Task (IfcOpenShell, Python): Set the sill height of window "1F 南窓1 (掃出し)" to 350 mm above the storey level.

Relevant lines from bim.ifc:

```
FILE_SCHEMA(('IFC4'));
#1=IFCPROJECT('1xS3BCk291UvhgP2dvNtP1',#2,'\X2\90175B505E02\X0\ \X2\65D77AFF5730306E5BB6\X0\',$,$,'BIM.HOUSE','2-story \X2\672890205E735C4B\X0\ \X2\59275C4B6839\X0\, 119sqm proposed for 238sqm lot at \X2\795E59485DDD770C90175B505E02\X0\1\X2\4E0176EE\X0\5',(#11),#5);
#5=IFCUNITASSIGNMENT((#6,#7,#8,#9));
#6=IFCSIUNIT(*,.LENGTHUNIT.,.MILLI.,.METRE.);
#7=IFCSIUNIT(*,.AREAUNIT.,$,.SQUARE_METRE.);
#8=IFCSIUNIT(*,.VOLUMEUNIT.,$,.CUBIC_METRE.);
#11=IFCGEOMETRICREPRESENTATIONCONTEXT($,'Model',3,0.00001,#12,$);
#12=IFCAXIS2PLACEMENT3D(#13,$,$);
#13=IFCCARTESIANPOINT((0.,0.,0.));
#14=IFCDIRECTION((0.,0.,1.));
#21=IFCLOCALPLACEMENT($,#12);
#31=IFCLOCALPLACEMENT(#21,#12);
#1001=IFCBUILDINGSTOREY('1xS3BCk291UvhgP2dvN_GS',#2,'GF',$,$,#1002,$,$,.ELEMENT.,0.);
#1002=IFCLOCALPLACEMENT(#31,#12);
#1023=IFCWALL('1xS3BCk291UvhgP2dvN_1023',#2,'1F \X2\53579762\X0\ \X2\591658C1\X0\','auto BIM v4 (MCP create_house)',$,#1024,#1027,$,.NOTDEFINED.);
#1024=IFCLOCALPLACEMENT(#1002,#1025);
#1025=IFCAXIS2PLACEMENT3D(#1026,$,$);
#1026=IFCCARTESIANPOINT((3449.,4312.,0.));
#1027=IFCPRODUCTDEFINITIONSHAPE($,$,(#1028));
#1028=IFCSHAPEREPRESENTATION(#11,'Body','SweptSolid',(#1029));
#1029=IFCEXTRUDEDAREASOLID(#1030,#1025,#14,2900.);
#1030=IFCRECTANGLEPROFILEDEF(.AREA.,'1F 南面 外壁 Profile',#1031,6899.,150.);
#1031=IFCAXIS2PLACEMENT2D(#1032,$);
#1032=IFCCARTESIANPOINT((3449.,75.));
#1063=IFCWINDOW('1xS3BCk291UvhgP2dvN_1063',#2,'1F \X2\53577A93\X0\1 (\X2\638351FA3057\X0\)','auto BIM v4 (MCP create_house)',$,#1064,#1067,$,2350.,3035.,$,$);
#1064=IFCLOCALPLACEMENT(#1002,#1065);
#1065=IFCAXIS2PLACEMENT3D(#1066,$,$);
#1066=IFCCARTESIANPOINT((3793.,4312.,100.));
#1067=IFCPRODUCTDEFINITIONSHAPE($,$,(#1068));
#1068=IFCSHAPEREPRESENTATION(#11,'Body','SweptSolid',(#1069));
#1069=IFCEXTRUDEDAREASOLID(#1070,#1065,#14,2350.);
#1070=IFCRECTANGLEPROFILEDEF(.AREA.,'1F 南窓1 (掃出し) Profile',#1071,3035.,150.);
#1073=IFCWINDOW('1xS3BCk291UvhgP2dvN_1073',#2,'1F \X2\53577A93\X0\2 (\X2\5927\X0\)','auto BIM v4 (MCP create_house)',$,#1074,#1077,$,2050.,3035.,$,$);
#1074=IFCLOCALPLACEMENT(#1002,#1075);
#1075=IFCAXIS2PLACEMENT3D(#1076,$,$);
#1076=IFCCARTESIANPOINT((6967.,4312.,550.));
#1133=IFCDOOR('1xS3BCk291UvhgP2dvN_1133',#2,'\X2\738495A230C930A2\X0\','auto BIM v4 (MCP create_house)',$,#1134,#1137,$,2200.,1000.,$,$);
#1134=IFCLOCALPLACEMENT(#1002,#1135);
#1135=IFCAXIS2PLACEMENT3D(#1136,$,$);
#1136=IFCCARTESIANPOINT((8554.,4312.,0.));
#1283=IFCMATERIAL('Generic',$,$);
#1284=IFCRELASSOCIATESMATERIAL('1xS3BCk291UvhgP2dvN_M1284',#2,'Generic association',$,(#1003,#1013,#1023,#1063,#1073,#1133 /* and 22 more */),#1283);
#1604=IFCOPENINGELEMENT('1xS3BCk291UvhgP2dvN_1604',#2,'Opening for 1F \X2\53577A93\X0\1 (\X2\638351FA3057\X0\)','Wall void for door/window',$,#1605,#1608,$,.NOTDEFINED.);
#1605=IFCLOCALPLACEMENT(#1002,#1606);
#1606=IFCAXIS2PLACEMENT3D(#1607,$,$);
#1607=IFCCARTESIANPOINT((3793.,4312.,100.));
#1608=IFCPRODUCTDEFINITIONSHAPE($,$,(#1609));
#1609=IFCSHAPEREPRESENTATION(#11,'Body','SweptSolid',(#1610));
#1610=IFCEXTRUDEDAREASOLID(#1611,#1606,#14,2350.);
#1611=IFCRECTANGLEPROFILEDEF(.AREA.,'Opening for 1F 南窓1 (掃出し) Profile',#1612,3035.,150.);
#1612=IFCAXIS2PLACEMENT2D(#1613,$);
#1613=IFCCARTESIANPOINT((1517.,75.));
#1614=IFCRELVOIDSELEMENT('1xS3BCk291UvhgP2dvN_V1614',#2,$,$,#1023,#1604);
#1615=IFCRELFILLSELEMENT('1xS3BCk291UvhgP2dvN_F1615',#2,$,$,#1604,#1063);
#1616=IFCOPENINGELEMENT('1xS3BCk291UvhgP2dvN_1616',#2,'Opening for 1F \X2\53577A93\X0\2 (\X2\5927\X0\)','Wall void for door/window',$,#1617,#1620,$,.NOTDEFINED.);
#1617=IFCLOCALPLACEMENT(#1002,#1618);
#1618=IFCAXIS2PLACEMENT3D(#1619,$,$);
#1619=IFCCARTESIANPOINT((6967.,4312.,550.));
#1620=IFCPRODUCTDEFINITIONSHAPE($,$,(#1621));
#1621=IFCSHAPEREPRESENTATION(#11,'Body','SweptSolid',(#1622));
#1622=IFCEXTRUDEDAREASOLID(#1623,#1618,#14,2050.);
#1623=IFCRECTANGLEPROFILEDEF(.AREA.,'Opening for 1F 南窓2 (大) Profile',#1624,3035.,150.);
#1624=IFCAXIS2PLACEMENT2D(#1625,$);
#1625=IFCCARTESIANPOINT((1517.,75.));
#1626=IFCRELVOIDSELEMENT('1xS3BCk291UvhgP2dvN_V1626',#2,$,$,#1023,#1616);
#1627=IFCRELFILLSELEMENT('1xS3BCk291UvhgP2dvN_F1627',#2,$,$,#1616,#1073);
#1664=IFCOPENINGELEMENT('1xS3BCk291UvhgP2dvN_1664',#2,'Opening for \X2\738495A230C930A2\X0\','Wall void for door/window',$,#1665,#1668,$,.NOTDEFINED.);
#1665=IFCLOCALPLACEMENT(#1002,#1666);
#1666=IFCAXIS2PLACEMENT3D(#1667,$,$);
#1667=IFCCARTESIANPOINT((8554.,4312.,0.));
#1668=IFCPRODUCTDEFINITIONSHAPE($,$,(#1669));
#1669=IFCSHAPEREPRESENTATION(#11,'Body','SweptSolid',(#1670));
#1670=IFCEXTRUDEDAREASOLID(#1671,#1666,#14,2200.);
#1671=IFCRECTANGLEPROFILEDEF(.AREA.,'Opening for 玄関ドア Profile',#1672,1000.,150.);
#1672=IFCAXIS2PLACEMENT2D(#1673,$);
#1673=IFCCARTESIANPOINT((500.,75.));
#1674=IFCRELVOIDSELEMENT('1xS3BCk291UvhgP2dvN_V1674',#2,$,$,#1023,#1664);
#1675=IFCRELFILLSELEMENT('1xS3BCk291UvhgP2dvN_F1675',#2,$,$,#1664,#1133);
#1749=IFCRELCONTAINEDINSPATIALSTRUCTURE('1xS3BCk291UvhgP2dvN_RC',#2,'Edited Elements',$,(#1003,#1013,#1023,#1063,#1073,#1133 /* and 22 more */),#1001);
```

```python
import numpy as np
import ifcopenshell
import ifcopenshell.api.geometry
import ifcopenshell.geom
import ifcopenshell.util.element
import ifcopenshell.util.placement
import ifcopenshell.util.shape
import ifcopenshell.util.unit

model = ifcopenshell.open("bim.ifc")
unit_scale = ifcopenshell.util.unit.calculate_unit_scale(model)

window = model.by_guid("1xS3BCk291UvhgP2dvN_1063")
opening = window.FillsVoids[0].RelatingOpeningElement
storey = ifcopenshell.util.element.get_container(window, ifc_class="IfcBuildingStorey")
level = ifcopenshell.util.placement.get_local_placement(storey.ObjectPlacement)[2, 3]

# The opening's origin need not be at the sill, so measure its lowest point.
shape = ifcopenshell.geom.create_shape(ifcopenshell.geom.settings(), opening)
bottom = ifcopenshell.util.shape.get_shape_bottom_elevation(shape, shape.geometry) / unit_scale
dz = level + 350.0 - bottom

shift = np.array([0.0, 0.0, dz])
# The window is not placed relative to its opening, so move both.
for product in (opening, window):
    matrix = ifcopenshell.util.placement.get_local_placement(product.ObjectPlacement)
    matrix[:3, 3] += shift
    ifcopenshell.api.geometry.edit_object_placement(model, product=product, matrix=matrix, is_si=False)

print(f"moved by {dz * unit_scale:+.3f} m")

model.write("bim_edited.ifc")
```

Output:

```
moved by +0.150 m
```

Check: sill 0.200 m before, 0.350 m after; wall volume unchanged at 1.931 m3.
